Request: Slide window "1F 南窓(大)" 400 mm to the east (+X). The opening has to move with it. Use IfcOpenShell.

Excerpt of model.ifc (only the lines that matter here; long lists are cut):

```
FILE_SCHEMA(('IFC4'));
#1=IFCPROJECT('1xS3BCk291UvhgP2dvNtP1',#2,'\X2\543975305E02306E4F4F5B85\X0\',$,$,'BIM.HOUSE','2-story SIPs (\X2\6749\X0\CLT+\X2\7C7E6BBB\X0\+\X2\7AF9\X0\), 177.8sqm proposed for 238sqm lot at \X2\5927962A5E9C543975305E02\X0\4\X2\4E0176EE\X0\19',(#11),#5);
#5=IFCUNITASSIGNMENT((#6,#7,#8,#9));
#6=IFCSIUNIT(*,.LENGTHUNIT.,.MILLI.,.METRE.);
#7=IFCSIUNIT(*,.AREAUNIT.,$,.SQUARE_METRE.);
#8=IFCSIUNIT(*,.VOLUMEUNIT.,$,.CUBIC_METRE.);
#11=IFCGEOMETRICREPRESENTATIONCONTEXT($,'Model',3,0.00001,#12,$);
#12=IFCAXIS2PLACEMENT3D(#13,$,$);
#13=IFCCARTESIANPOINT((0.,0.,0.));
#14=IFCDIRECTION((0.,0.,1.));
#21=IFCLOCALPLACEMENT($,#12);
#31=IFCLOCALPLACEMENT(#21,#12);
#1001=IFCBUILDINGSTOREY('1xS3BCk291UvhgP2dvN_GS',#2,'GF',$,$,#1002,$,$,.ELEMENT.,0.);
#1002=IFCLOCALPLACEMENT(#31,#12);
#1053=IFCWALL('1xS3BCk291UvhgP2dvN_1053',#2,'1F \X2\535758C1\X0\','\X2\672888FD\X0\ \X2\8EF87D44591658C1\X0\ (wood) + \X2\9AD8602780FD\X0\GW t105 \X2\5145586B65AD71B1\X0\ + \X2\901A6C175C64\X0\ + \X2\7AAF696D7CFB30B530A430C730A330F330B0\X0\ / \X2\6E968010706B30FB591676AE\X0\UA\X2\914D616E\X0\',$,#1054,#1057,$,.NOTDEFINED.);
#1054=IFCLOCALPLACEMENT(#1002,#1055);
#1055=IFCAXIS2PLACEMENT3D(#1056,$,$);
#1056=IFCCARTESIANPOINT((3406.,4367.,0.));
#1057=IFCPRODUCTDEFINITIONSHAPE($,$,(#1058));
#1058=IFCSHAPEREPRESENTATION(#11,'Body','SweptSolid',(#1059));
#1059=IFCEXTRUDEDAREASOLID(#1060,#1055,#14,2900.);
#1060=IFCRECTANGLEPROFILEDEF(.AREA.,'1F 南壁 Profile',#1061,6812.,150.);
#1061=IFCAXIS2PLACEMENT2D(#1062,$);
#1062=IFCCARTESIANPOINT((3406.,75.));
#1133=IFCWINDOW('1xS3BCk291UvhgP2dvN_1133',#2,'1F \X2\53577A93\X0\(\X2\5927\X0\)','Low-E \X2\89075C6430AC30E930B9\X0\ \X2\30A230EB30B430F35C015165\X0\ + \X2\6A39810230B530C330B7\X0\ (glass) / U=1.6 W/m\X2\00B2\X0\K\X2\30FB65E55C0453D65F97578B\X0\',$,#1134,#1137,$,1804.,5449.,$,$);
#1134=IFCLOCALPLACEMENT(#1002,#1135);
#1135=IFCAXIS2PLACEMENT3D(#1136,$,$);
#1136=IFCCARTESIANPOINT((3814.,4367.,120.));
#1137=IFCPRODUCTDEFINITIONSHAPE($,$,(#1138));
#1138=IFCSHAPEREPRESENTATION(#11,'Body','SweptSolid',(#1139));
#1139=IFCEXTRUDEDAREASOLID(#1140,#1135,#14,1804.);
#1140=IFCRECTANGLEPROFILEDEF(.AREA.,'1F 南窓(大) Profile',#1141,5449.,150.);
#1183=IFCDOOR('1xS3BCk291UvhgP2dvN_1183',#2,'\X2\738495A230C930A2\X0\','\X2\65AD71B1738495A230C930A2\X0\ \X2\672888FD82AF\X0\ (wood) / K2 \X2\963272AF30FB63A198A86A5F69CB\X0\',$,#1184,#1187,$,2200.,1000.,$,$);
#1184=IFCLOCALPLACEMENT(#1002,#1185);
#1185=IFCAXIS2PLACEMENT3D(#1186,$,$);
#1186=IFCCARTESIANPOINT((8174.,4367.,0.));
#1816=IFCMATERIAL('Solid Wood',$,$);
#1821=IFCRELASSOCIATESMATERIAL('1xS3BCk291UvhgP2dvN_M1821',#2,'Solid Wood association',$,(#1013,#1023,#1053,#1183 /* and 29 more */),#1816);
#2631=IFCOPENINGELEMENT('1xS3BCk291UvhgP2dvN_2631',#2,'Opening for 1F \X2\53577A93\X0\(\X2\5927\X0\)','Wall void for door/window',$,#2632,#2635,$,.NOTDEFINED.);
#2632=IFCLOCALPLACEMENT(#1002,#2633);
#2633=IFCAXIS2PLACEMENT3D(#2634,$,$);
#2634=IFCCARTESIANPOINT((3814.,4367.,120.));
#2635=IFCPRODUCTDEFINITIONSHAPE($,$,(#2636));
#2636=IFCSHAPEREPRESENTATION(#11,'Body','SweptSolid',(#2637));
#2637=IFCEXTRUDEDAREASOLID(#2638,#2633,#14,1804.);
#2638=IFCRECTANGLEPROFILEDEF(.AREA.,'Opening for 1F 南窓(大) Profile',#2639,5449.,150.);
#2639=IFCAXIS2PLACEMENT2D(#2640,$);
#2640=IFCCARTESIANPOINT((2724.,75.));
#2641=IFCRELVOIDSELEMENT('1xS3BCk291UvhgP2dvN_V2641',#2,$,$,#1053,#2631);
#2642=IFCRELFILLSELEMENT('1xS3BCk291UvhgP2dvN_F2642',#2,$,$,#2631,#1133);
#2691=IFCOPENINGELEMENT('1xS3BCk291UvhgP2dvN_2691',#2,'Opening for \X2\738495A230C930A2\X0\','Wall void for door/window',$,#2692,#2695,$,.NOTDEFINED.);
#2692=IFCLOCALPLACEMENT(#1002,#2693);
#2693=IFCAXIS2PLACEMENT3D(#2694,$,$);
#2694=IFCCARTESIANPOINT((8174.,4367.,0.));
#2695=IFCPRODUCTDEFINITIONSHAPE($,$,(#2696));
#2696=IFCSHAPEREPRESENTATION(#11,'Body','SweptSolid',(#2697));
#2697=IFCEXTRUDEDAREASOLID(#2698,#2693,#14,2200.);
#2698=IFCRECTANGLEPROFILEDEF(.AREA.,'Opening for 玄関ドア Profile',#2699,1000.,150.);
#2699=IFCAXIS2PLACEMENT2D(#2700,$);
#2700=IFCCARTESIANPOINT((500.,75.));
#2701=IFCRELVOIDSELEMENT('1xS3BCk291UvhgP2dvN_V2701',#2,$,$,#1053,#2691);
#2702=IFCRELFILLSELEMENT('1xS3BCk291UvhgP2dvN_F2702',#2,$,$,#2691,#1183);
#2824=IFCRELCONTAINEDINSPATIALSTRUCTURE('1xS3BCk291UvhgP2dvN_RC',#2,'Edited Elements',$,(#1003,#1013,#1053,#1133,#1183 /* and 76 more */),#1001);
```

```python
import ifcopenshell
import ifcopenshell.api.geometry
import ifcopenshell.util.placement

model = ifcopenshell.open("model.ifc")

window = model.by_guid("1xS3BCk291UvhgP2dvN_1133")
opening = window.FillsVoids[0].RelatingOpeningElement
wall = opening.VoidsElements[0].RelatingBuildingElement

wall_matrix = ifcopenshell.util.placement.get_local_placement(wall.ObjectPlacement)
shift = wall_matrix[:3, 0] * 400.0
before = ifcopenshell.util.placement.get_local_placement(window.ObjectPlacement)[:3, 3].copy()

# The window is not placed relative to its opening, so move both.
for product in (opening, window):
    matrix = ifcopenshell.util.placement.get_local_placement(product.ObjectPlacement)
    matrix[:3, 3] += shift
    ifcopenshell.api.geometry.edit_object_placement(model, product=product, matrix=matrix, is_si=False)

after = ifcopenshell.util.placement.get_local_placement(window.ObjectPlacement)[:3, 3]
print("window moved by", (after - before).round(3) + 0.0)

model.write("model_v2.ifc")
```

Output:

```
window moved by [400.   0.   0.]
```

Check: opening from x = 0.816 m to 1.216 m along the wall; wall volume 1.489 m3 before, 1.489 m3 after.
